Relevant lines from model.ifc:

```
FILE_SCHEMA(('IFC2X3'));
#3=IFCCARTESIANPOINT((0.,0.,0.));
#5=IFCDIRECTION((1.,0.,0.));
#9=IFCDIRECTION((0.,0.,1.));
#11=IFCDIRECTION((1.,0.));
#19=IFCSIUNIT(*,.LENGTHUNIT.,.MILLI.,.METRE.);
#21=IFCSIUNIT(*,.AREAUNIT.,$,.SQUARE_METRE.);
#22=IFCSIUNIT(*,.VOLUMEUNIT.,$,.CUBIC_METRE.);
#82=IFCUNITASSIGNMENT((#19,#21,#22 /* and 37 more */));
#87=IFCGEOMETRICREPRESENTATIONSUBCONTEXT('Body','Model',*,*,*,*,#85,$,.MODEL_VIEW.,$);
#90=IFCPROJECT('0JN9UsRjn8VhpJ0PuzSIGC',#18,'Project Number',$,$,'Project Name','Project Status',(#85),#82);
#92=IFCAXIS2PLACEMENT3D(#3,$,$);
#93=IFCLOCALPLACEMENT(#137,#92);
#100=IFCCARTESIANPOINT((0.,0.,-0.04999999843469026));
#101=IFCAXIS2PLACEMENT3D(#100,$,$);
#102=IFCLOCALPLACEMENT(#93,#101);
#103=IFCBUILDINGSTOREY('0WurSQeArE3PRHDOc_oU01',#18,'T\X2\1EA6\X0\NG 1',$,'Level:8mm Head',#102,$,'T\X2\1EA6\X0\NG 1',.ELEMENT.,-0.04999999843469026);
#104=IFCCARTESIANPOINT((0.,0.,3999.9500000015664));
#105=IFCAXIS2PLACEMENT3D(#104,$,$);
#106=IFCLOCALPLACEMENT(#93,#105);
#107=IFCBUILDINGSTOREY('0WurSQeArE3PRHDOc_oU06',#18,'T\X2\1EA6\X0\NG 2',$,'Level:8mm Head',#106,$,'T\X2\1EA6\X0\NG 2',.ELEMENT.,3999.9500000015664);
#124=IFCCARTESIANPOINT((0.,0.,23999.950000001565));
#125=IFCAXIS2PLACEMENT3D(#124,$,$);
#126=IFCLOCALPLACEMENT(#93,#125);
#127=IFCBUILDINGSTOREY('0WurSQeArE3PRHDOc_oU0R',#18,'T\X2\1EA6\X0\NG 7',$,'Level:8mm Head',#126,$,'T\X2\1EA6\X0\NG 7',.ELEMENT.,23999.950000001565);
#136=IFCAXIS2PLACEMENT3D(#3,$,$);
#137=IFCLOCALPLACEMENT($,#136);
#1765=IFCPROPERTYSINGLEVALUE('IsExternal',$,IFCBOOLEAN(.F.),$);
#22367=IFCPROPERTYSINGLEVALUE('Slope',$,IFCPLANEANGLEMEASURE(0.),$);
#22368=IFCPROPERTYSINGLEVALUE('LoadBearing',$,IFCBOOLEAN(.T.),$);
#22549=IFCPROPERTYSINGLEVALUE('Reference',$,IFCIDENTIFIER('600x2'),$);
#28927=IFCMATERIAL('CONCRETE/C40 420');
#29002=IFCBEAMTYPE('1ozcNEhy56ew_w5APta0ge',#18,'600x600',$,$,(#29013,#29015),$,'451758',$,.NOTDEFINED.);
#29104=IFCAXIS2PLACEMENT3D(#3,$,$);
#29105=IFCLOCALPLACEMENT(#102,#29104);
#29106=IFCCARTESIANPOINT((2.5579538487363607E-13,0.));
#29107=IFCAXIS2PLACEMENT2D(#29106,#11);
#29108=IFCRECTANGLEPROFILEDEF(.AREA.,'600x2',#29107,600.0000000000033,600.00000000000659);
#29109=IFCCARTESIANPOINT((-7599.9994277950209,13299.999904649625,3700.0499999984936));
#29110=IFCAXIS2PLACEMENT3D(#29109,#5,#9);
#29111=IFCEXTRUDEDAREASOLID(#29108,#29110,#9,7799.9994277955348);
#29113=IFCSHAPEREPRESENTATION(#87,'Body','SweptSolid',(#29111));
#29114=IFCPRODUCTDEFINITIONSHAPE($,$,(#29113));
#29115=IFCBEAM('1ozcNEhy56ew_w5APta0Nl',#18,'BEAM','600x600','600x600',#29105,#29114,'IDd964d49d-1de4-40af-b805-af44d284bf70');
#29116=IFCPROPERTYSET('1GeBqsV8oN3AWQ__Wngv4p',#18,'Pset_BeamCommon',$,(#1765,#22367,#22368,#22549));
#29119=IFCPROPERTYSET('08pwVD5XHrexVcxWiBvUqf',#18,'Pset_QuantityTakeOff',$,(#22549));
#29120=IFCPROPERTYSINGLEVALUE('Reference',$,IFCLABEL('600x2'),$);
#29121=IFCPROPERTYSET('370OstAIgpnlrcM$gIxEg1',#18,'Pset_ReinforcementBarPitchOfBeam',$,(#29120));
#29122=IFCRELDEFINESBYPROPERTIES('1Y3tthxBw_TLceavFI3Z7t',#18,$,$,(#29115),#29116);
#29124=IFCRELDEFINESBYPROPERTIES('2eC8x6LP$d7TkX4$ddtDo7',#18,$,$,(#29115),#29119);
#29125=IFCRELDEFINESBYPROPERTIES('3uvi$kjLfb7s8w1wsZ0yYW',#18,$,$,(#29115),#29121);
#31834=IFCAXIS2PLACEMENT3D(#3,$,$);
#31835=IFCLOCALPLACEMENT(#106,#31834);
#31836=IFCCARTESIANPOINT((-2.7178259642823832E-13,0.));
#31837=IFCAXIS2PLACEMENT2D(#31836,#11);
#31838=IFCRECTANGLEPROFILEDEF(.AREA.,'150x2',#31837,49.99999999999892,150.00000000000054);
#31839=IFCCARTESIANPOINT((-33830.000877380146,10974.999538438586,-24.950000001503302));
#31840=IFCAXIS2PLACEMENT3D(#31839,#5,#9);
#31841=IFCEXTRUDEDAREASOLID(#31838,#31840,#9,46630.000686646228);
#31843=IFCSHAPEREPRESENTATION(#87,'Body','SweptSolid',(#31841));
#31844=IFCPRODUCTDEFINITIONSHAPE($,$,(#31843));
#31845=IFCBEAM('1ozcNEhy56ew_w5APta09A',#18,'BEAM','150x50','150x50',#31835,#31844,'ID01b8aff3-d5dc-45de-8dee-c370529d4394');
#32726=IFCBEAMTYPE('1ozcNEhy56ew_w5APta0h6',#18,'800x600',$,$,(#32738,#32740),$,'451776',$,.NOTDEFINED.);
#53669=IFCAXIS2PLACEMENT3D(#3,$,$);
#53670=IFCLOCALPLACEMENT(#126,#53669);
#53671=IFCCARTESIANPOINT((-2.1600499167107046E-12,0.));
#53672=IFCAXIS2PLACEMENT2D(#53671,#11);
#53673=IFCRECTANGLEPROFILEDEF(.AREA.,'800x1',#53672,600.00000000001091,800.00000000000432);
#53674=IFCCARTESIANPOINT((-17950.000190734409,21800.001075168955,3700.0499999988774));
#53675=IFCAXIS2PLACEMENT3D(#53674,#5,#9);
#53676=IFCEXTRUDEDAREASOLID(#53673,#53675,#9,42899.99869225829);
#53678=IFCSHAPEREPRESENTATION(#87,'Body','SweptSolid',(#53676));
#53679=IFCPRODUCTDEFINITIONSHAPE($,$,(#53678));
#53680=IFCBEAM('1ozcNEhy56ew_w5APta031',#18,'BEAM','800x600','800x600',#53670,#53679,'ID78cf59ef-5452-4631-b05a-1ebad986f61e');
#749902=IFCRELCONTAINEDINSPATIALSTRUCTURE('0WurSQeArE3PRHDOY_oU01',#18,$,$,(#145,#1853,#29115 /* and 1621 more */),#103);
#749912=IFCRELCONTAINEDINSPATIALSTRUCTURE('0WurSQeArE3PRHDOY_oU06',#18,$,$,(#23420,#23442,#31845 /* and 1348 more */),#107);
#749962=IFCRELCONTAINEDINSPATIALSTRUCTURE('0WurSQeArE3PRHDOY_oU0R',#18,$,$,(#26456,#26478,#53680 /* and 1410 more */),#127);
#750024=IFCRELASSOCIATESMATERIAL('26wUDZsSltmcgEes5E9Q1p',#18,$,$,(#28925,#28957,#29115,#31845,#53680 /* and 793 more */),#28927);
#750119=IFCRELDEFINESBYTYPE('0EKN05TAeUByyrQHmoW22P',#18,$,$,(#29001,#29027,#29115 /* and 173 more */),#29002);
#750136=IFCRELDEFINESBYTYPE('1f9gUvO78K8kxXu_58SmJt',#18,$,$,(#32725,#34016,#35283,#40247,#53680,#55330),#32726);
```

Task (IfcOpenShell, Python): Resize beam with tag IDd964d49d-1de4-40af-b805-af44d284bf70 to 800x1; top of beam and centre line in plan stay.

```python
import ifcopenshell
import ifcopenshell.api.pset
import ifcopenshell.api.type
import ifcopenshell.util.element
import ifcopenshell.util.representation

model = ifcopenshell.open("model.ifc")

member = model.by_guid("1ozcNEhy56ew_w5APta0Nl")
source = next(p for p in model.by_type("IfcRectangleProfileDef") if p.ProfileName == "800x1")

body = ifcopenshell.util.representation.get_representation(member, "Model", "Body")
solid = body.Items[0]
old_profile = solid.SweptArea

# Copy the section's sizes but keep this member's own profile position.
profile = ifcopenshell.util.element.copy(model, source)
# Profiles are centred, so shift by half the change in depth to hold the top.
shift = (old_profile.XDim - profile.XDim) / 2
x, y = old_profile.Position.Location.Coordinates
up = (1.0, 0.0)  # upwards, in the solid's own plane
location = model.createIfcCartesianPoint((x + up[0] * shift, y + up[1] * shift))
profile.Position = model.createIfcAxis2Placement2D(location, old_profile.Position.RefDirection)
solid.SweptArea = profile
if not model.get_total_inverses(old_profile):
    ifcopenshell.util.element.remove_deep2(model, old_profile)

new_type = model.by_id(32726)
ifcopenshell.api.type.assign_type(
    model, related_objects=[member], relating_type=new_type, should_map_representations=False
)
member.Description = "800x600"
member.ObjectType = "800x600"
pset = model.by_id(ifcopenshell.util.element.get_pset(member, "Pset_BeamCommon", should_inherit=False)["id"])
ifcopenshell.api.pset.edit_pset(model, pset=pset, properties={"Reference": "800x1"})
pset = model.by_id(ifcopenshell.util.element.get_pset(member, "Pset_QuantityTakeOff", should_inherit=False)["id"])
ifcopenshell.api.pset.edit_pset(model, pset=pset, properties={"Reference": "800x1"})
pset = model.by_id(ifcopenshell.util.element.get_pset(member, "Pset_ReinforcementBarPitchOfBeam", should_inherit=False)["id"])
ifcopenshell.api.pset.edit_pset(model, pset=pset, properties={"Reference": "800x1"})

print(solid.SweptArea)

model.write("model_updated.ifc")
```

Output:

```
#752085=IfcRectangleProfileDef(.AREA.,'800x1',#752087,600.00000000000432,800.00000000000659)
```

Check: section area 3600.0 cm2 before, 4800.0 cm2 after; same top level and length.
